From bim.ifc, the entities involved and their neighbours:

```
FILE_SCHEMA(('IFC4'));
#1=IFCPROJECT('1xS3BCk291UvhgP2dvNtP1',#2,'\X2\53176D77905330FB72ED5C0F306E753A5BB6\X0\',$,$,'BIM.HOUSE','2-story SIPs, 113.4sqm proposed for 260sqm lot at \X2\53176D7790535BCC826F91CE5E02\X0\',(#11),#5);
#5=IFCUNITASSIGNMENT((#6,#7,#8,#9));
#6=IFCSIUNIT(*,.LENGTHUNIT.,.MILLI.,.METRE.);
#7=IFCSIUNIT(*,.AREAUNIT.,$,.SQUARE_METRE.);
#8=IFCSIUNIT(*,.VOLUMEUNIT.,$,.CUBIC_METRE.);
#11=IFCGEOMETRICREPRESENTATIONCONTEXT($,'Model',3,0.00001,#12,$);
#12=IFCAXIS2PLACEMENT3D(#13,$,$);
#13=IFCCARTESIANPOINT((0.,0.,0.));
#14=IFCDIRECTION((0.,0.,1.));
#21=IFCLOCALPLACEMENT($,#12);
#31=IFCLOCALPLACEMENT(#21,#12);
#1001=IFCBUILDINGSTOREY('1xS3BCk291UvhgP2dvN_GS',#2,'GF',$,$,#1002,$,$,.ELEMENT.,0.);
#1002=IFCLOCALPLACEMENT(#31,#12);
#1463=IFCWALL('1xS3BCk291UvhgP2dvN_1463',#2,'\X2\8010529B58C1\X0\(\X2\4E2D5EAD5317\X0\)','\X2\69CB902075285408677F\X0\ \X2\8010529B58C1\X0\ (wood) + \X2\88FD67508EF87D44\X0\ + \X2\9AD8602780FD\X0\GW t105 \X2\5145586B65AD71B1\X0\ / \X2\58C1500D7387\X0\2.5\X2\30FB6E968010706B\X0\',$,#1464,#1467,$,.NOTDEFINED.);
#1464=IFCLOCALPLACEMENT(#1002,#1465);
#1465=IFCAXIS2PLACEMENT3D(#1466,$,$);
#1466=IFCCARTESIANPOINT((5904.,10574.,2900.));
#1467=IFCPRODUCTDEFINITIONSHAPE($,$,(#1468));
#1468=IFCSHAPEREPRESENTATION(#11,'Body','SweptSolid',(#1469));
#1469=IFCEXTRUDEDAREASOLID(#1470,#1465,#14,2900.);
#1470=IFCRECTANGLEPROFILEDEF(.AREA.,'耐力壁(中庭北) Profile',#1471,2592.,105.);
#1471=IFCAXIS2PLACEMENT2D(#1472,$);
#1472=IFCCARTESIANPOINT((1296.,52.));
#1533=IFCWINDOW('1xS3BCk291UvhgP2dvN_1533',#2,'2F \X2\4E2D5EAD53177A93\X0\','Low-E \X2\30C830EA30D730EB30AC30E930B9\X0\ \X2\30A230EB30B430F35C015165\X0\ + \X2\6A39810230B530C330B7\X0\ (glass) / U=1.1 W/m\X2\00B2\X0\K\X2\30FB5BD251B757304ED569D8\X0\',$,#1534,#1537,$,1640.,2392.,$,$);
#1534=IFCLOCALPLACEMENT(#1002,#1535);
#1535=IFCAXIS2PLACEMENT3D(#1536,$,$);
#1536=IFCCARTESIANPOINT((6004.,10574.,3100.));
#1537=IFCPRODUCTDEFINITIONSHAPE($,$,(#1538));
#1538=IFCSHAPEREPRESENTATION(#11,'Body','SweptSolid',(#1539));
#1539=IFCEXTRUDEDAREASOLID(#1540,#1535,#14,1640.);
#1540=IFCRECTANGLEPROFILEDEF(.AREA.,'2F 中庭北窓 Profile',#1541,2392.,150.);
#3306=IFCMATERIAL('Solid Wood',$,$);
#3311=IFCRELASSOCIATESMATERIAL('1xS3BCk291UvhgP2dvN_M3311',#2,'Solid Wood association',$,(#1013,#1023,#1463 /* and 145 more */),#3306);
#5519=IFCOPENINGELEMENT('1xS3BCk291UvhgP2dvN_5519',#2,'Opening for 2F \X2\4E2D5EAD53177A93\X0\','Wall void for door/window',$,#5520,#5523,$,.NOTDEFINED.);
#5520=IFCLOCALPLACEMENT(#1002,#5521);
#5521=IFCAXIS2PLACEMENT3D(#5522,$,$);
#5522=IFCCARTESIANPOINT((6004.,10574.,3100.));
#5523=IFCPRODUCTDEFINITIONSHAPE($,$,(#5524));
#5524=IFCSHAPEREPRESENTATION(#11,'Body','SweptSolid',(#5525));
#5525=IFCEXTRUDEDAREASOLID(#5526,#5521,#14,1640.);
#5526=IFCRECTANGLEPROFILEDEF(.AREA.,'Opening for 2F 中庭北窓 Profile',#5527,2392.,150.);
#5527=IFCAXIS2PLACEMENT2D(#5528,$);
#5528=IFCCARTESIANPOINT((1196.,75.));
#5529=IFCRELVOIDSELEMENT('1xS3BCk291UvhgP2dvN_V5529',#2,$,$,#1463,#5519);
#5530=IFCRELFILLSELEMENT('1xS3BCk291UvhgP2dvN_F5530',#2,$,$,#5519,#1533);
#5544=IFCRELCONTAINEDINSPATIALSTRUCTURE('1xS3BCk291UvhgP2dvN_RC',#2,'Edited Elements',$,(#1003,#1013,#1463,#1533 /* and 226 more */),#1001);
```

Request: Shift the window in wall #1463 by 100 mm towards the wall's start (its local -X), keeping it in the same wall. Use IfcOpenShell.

```python
import ifcopenshell
import ifcopenshell.api.geometry
import ifcopenshell.util.placement

model = ifcopenshell.open("bim.ifc")

window = model.by_id(1533)
opening = window.FillsVoids[0].RelatingOpeningElement
wall = opening.VoidsElements[0].RelatingBuildingElement

wall_matrix = ifcopenshell.util.placement.get_local_placement(wall.ObjectPlacement)
shift = wall_matrix[:3, 0] * -100.0
before = ifcopenshell.util.placement.get_local_placement(window.ObjectPlacement)[:3, 3].copy()

# The window is not placed relative to its opening, so move both.
for product in (opening, window):
    matrix = ifcopenshell.util.placement.get_local_placement(product.ObjectPlacement)
    matrix[:3, 3] += shift
    ifcopenshell.api.geometry.edit_object_placement(model, product=product, matrix=matrix, is_si=False)

after = ifcopenshell.util.placement.get_local_placement(window.ObjectPlacement)[:3, 3]
print("window moved by", (after - before).round(3) + 0.0)

model.write("bim-out.ifc")
```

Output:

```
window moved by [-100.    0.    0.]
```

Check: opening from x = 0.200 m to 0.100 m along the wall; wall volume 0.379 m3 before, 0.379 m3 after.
